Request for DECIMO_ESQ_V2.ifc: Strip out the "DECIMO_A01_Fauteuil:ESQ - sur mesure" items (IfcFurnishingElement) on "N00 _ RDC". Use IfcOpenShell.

First a look at what the model holds.

```python
import ifcopenshell
import ifcopenshell.util.element

model = ifcopenshell.open("DECIMO_ESQ_V2.ifc")
print(model.schema)
storey = next(s for s in model.by_type("IfcBuildingStorey") if s.Name == "N00 _ RDC")
furniture = [e for e in ifcopenshell.util.element.get_decomposition(storey) if e.is_a("IfcFurnishingElement")]
seen = {}
for e in furniture:
    element_type = ifcopenshell.util.element.get_type(e)
    name = element_type.Name if element_type not in (None, e) else None
    seen[name] = seen.get(name, 0) + 1
for name, count in sorted(seen.items(), key=str):
    print(count, "x", name)
```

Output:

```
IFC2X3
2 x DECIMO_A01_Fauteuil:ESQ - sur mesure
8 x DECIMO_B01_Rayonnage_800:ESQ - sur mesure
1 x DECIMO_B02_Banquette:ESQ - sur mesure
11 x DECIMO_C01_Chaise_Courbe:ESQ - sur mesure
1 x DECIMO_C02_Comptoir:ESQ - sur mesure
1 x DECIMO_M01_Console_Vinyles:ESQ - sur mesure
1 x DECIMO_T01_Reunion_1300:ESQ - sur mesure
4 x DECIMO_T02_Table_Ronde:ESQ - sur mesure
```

```python
import ifcopenshell
import ifcopenshell.api.root
import ifcopenshell.util.element

model = ifcopenshell.open("DECIMO_ESQ_V2.ifc")

storey = next(s for s in model.by_type("IfcBuildingStorey") if s.Name == "N00 _ RDC")
furniture = [e for e in ifcopenshell.util.element.get_decomposition(storey) if e.is_a("IfcFurnishingElement")]
targets = [e for e in furniture if (t := ifcopenshell.util.element.get_type(e)) not in (None, e) and t.Name == "DECIMO_A01_Fauteuil:ESQ - sur mesure"]

for e in targets:
    ifcopenshell.api.root.remove_product(model, product=e)
print(len(targets), "removed")

model.write("DECIMO_ESQ_V2_edited.ifc")
```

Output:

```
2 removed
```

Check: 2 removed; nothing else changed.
